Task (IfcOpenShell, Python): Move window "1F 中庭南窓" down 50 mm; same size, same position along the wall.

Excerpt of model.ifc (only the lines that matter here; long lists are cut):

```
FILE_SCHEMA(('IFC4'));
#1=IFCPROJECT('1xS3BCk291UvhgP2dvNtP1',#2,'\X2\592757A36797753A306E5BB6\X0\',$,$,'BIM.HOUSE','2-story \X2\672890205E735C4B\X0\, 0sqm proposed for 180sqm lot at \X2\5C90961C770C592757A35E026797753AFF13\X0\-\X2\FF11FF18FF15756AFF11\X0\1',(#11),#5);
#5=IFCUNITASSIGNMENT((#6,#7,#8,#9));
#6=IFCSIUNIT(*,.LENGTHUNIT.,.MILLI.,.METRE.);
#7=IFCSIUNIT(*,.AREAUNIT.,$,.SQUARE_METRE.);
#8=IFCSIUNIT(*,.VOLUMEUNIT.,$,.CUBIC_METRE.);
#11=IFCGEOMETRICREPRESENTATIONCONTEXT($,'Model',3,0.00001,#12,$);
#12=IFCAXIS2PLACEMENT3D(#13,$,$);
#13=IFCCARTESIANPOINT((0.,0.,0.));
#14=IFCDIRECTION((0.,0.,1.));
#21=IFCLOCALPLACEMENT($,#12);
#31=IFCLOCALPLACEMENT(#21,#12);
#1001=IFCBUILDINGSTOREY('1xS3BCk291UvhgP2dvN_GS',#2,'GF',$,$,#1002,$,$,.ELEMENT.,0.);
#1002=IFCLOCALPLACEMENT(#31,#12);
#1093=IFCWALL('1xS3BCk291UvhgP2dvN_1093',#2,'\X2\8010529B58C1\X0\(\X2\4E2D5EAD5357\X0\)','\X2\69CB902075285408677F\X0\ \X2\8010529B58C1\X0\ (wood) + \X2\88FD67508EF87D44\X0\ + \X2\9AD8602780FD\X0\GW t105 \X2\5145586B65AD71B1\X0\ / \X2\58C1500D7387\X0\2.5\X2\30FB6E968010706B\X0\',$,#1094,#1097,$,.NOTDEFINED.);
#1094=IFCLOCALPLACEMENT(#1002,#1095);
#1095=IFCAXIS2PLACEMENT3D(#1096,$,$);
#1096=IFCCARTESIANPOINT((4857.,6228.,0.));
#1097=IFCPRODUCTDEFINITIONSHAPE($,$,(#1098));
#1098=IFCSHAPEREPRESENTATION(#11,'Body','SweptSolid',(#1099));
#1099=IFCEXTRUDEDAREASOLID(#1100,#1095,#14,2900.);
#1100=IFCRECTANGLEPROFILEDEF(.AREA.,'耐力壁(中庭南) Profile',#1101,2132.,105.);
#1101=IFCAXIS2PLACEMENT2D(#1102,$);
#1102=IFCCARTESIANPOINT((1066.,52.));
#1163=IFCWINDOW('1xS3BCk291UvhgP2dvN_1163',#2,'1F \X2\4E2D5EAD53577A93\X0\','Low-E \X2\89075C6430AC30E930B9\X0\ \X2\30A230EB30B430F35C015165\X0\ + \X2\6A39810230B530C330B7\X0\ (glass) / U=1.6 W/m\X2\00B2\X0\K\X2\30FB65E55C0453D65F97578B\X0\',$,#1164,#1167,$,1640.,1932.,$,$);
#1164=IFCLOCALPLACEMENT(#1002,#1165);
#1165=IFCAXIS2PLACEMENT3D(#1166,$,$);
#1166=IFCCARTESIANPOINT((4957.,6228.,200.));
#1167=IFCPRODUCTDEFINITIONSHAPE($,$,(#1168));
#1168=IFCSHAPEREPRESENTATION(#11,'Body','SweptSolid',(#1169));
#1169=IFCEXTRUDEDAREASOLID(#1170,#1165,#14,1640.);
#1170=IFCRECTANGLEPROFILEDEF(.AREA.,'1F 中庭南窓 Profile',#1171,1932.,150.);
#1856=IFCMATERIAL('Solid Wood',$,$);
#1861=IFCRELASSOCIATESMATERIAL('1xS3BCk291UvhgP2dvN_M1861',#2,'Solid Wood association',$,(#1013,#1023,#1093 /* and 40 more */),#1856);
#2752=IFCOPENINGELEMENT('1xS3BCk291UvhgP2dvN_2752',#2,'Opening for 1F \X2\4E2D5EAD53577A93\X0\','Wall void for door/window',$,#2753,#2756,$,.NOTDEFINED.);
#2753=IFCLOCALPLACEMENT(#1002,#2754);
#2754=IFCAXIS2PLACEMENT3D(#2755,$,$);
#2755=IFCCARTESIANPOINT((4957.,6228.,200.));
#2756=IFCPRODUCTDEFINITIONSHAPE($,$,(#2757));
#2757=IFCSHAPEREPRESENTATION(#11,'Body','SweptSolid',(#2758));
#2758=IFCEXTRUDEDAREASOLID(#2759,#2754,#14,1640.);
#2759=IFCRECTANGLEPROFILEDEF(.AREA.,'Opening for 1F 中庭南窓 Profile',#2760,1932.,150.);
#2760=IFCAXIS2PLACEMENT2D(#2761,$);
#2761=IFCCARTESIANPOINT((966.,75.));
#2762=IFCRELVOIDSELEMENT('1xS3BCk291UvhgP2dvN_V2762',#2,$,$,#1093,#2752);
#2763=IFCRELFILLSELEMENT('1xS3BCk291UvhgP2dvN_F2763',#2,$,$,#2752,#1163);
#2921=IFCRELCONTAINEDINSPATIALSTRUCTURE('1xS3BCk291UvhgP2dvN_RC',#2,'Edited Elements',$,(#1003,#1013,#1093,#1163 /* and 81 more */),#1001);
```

```python
import numpy as np
import ifcopenshell
import ifcopenshell.api.geometry
import ifcopenshell.util.placement
import ifcopenshell.util.unit

model = ifcopenshell.open("model.ifc")
unit_scale = ifcopenshell.util.unit.calculate_unit_scale(model)

window = model.by_guid("1xS3BCk291UvhgP2dvN_1163")
opening = window.FillsVoids[0].RelatingOpeningElement
dz = -0.05 / unit_scale

shift = np.array([0.0, 0.0, dz])
# The window is not placed relative to its opening, so move both.
for product in (opening, window):
    matrix = ifcopenshell.util.placement.get_local_placement(product.ObjectPlacement)
    matrix[:3, 3] += shift
    ifcopenshell.api.geometry.edit_object_placement(model, product=product, matrix=matrix, is_si=False)

print(f"moved by {dz * unit_scale:+.3f} m")

model.write("model_v2.ifc")
```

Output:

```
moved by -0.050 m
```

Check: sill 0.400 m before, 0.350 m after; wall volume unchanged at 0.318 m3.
